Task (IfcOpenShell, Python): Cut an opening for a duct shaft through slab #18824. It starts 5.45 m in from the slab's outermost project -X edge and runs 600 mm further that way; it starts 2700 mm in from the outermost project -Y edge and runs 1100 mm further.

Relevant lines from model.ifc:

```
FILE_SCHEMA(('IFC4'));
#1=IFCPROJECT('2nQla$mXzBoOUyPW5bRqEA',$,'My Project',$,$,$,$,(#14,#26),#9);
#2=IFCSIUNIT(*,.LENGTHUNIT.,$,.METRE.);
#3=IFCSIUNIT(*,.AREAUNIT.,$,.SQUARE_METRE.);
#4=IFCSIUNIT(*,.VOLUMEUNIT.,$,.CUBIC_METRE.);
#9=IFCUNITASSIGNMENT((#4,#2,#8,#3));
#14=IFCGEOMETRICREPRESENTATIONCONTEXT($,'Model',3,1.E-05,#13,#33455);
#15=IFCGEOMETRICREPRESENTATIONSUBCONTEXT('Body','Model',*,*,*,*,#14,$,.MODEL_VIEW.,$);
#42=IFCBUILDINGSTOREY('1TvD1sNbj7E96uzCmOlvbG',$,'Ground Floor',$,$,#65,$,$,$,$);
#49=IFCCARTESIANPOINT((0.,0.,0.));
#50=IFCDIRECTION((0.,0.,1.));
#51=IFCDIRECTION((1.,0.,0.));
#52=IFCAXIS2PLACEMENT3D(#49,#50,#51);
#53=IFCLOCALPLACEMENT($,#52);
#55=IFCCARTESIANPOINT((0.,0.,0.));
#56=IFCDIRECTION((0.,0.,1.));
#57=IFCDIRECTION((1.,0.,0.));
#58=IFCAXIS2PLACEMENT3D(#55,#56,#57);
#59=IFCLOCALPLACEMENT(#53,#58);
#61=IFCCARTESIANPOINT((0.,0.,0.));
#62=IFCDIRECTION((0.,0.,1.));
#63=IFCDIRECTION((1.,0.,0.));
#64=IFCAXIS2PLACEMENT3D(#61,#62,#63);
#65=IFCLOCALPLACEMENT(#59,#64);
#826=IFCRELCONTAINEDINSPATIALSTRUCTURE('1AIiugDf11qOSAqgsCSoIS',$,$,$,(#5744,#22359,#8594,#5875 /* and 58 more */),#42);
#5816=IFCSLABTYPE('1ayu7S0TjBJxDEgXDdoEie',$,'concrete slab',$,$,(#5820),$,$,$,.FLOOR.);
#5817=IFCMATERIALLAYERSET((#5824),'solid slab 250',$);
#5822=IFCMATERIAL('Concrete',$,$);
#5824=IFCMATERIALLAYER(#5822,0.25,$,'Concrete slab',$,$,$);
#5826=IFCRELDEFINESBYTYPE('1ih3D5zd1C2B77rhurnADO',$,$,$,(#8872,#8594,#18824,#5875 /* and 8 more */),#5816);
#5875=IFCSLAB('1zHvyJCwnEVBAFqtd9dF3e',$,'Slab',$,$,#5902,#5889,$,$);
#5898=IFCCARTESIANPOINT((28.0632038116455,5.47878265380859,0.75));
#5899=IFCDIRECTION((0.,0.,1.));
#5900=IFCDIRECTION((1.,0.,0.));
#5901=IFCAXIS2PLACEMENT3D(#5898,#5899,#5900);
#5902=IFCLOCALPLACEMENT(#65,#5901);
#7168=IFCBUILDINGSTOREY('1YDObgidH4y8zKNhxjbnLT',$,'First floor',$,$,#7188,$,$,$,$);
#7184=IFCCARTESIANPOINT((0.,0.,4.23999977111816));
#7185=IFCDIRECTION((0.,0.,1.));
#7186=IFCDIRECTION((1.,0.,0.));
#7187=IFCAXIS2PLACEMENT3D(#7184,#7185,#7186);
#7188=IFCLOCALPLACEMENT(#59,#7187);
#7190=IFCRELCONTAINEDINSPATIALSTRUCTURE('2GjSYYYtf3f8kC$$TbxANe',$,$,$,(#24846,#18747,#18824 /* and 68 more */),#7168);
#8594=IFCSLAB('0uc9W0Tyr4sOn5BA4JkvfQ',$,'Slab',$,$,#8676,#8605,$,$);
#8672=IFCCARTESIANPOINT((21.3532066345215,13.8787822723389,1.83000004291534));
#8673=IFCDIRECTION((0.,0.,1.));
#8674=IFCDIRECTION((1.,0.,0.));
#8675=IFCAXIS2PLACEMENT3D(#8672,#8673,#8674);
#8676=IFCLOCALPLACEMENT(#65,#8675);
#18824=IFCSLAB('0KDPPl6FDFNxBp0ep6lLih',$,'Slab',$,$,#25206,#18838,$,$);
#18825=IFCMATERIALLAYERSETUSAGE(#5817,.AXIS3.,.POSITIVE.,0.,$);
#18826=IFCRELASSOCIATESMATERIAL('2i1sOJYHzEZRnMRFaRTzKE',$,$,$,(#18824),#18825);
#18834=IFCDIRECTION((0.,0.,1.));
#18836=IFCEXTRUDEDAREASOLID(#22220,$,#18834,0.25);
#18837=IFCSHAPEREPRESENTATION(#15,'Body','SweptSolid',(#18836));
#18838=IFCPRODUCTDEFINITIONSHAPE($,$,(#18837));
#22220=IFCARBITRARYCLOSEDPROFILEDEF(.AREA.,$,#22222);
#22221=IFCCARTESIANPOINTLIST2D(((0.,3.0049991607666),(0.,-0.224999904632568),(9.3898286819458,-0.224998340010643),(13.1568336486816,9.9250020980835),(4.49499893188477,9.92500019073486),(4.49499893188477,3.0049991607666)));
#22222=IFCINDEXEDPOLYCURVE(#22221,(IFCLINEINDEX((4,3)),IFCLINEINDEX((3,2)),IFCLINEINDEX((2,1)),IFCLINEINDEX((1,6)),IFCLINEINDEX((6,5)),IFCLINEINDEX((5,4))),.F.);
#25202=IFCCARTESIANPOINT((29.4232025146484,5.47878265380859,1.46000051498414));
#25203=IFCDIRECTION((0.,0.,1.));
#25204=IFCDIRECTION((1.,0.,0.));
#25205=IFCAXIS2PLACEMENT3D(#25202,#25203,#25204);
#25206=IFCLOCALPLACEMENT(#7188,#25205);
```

```python
import numpy as np
import ifcopenshell
import ifcopenshell.api.feature
import ifcopenshell.api.geometry
import ifcopenshell.api.root
import ifcopenshell.geom
import ifcopenshell.util.placement
import ifcopenshell.util.representation
import ifcopenshell.util.shape
import ifcopenshell.util.unit

model = ifcopenshell.open("model.ifc")
unit_scale = ifcopenshell.util.unit.calculate_unit_scale(model)
settings = ifcopenshell.geom.settings()


def volume(element):
    """Net volume in cubic metres, openings subtracted."""
    shape = ifcopenshell.geom.create_shape(settings, element)
    return ifcopenshell.util.shape.get_volume(shape.geometry)


slab = model.by_id(18824)
before = volume(slab)

# Extent in the slab's own axes, in metres. The edges named are its -X and -Y sides.
slab_shape = ifcopenshell.geom.create_shape(settings, slab)
vertices = ifcopenshell.util.shape.get_vertices(slab_shape.geometry)
x_min, y_min, bottom = vertices.min(axis=0)
top = vertices[:, 2].max()

opening = ifcopenshell.api.root.create_entity(model, ifc_class="IfcOpeningElement", name="Duct shaft opening", predefined_type="OPENING")
context = ifcopenshell.util.representation.get_context(model, "Model", "Body", "MODEL_VIEW")
width, depth = 0.6, 1.1
outline = [(0.0, 0.0), (width, 0.0), (width, depth), (0.0, depth), (0.0, 0.0)]
# Overshoot both faces by 50 mm so the cut is clean.
shape = ifcopenshell.api.geometry.add_slab_representation(
    model, context=context, depth=top - bottom + 0.1, polyline=outline
)
ifcopenshell.api.geometry.assign_representation(model, product=opening, representation=shape)

matrix = ifcopenshell.util.placement.get_local_placement(slab.ObjectPlacement)
matrix[:, 3] = matrix @ np.append(np.array([x_min + 5.45, y_min + 2.7, bottom - 0.05]) / unit_scale, 1.0)
ifcopenshell.api.geometry.edit_object_placement(model, product=opening, matrix=matrix, is_si=False)
ifcopenshell.api.feature.add_feature(model, feature=opening, element=slab)

after = volume(slab)

print(f"slab volume {before:.3f} -> {after:.3f} m3")

model.write("model_updated.ifc")
```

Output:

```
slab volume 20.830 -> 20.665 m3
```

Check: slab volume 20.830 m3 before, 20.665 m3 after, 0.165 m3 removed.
